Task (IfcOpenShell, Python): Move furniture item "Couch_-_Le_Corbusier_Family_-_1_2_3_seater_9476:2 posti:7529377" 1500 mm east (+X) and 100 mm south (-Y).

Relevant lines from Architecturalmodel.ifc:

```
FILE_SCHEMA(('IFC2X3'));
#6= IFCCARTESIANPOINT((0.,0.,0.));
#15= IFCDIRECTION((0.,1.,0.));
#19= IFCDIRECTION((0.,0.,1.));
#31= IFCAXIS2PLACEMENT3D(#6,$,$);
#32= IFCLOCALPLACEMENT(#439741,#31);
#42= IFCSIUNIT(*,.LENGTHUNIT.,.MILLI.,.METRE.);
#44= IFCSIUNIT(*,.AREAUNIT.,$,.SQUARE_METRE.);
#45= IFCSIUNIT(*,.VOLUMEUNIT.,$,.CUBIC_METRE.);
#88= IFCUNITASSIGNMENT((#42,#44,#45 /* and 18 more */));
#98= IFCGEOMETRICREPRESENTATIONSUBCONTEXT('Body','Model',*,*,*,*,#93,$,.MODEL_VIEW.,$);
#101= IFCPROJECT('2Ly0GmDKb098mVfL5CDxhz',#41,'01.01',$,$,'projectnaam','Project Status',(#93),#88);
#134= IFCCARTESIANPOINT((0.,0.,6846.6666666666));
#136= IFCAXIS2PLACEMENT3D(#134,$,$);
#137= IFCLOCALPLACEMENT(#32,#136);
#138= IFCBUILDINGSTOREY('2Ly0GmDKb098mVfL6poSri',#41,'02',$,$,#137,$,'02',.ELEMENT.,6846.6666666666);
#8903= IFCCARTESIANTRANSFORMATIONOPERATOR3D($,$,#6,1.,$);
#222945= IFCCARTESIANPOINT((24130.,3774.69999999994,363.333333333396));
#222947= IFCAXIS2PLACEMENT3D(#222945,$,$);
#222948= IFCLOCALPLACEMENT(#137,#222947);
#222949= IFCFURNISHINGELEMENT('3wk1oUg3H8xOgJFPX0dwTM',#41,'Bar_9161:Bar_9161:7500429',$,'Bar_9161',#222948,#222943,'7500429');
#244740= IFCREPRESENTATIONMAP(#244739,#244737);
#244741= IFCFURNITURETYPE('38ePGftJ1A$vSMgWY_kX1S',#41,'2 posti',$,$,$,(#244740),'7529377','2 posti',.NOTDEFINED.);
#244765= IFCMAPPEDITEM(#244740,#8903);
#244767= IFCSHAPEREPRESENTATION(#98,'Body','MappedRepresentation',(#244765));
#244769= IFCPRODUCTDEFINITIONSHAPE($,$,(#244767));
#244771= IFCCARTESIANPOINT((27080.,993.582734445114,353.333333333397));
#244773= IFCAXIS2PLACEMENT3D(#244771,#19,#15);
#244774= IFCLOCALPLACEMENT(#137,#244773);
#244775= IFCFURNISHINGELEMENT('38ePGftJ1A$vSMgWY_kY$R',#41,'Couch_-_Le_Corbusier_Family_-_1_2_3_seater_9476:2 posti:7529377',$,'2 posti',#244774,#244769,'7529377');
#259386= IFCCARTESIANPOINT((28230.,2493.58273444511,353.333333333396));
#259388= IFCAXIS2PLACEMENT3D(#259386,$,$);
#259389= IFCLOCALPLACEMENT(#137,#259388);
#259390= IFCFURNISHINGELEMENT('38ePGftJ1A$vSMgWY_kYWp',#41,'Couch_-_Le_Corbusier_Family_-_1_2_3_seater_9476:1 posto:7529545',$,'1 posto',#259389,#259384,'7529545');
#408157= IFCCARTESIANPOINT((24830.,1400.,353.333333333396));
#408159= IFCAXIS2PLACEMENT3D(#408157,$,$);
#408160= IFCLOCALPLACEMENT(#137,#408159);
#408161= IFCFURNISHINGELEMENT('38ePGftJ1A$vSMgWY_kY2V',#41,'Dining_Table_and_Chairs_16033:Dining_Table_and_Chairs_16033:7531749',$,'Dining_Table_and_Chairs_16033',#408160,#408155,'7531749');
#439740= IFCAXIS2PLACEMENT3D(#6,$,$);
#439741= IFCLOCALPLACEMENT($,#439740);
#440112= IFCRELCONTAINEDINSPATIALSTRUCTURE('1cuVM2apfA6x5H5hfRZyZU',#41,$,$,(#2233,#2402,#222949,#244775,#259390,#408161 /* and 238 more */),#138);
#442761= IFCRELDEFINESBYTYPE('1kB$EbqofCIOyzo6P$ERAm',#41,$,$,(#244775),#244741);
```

```python
import ifcopenshell
import ifcopenshell.api.geometry
import ifcopenshell.util.placement

model = ifcopenshell.open("Architecturalmodel.ifc")

item = model.by_guid("38ePGftJ1A$vSMgWY_kY$R")
matrix = ifcopenshell.util.placement.get_local_placement(item.ObjectPlacement)
matrix[0, 3] += 1500.0
matrix[1, 3] -= 100.0
ifcopenshell.api.geometry.edit_object_placement(model, product=item, matrix=matrix, is_si=False)

print(ifcopenshell.util.placement.get_local_placement(item.ObjectPlacement).round(3) + 0.0)

model.write("Architecturalmodel_updated.ifc")
```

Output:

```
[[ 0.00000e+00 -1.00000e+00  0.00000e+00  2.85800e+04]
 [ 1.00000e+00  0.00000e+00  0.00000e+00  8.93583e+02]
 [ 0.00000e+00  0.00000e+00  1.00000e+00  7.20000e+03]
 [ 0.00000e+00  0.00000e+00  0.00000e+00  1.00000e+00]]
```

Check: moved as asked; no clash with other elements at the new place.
